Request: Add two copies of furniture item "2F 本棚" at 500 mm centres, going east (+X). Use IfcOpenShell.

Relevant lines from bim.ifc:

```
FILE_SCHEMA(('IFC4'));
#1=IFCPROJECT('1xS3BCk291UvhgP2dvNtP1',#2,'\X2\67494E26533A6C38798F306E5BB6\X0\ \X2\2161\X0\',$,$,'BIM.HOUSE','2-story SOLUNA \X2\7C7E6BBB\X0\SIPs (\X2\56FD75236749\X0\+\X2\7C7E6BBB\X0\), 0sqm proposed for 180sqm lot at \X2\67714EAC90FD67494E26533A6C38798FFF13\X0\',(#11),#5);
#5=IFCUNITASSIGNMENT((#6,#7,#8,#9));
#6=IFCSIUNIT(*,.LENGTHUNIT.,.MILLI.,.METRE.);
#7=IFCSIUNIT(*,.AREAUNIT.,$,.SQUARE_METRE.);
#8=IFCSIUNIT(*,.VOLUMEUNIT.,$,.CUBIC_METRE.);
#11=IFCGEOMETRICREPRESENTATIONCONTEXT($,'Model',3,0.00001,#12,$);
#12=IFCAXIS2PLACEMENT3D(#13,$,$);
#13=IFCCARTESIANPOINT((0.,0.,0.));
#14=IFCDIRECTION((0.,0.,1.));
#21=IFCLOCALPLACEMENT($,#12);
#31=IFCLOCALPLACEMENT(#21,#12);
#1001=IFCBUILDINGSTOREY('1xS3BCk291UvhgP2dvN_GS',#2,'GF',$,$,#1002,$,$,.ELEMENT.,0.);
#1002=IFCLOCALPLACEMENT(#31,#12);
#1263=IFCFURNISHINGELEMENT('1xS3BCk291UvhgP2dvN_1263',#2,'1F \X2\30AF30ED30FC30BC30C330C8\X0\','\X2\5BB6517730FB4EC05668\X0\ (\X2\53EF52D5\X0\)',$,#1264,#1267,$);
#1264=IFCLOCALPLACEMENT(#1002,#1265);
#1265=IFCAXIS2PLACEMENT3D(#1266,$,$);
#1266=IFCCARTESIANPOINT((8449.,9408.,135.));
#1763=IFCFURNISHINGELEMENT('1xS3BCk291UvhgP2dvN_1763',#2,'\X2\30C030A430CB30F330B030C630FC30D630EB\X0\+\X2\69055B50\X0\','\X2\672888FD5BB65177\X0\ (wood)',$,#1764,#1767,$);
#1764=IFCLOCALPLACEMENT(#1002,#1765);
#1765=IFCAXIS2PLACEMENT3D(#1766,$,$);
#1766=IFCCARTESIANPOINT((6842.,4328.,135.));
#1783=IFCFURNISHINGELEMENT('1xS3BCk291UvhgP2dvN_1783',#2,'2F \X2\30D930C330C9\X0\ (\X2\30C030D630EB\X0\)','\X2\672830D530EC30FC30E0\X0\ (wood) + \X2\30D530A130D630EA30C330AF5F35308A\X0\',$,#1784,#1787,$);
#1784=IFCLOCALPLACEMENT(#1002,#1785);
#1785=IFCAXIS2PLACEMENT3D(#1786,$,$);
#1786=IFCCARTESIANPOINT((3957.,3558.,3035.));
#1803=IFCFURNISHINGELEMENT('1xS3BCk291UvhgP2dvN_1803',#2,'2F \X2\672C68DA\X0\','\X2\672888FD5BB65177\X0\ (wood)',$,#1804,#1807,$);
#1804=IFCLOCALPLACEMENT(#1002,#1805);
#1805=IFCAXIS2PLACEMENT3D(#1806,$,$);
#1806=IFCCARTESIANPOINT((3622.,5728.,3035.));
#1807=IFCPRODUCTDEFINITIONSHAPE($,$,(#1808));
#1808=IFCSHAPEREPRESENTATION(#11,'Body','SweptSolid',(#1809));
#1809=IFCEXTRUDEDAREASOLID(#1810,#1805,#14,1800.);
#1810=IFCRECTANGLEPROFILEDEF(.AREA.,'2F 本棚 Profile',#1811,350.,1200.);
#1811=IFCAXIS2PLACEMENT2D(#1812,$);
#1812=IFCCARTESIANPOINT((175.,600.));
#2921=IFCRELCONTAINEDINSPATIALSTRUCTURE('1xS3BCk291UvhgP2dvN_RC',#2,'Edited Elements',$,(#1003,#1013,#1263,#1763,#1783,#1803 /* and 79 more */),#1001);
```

```python
import numpy as np
import ifcopenshell
import ifcopenshell.api.geometry
import ifcopenshell.api.root
import ifcopenshell.util.element
import ifcopenshell.util.placement
import ifcopenshell.util.unit

model = ifcopenshell.open("bim.ifc")
unit_scale = ifcopenshell.util.unit.calculate_unit_scale(model)


def reuse_history(source, copy):
    """copy_class also copies each property set's owner history, people and application; keep the originals."""
    for rel in copy.IsDefinedBy:
        if rel.is_a("IfcRelDefinesByProperties") and (history := rel.RelatingPropertyDefinition.OwnerHistory):
            rel.RelatingPropertyDefinition.OwnerHistory = source.OwnerHistory
            ifcopenshell.util.element.remove_deep2(model, history)


source = model.by_id(1803)
base = ifcopenshell.util.placement.get_local_placement(source.ObjectPlacement)
step = np.array([1.0, 0.0, 0.0]) * 0.5 / unit_scale

for i in range(1, 3):
    copy = ifcopenshell.api.root.copy_class(model, product=source)
    copy.Representation = ifcopenshell.util.element.copy_deep(
        model, source.Representation, exclude=["IfcGeometricRepresentationContext", "IfcRepresentationMap"]
    )
    reuse_history(source, copy)
    matrix = base.copy()
    matrix[:3, 3] += i * step
    print("added at", matrix[:3, 3].round(3) + 0.0)
    ifcopenshell.api.geometry.edit_object_placement(model, product=copy, matrix=matrix, is_si=False)

model.write("bim_edited.ifc")
```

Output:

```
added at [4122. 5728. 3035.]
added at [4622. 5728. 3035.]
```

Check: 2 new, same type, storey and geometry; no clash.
